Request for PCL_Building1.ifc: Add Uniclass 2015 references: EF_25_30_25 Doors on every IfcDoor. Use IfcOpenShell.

First a look at what the model holds.

```python
import ifcopenshell

model = ifcopenshell.open("PCL_Building1.ifc")
print(model.schema)
print("classifications:", [c.Name for c in model.by_type("IfcClassification")])
for ifc_class in ("IfcDoor", "IfcRoof", "IfcStair", "IfcWall", "IfcWindow"):
    print(ifc_class, len(model.by_type(ifc_class)))
```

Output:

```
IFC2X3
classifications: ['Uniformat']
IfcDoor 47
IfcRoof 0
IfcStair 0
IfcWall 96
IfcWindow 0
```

```python
import ifcopenshell
import ifcopenshell.api.classification

model = ifcopenshell.open("PCL_Building1.ifc")

# IFC2X3 requires Source and Edition and has no link from the project to the system.
system = model.create_entity("IfcClassification", Source="NBS", Edition="2015", Name="Uniclass 2015")

codes = {
    "IfcDoor": ("EF_25_30_25", "Doors"),
}
for ifc_class, (code, name) in codes.items():
    products = model.by_type(ifc_class)
    ifcopenshell.api.classification.add_reference(
        model, products=products, classification=system, identification=code, name=name
    )
    print(code, len(products))

model.write("PCL_Building1-out.ifc")
```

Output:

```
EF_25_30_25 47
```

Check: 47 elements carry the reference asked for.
